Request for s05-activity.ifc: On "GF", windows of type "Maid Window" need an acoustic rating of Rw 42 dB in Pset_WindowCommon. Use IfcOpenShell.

First a look at what the model holds.

```python
import ifcopenshell
import ifcopenshell.util.element

model = ifcopenshell.open("s05-activity.ifc")
print(model.schema)
storey = next(s for s in model.by_type("IfcBuildingStorey") if s.Name == "GF")
windows = [e for e in ifcopenshell.util.element.get_decomposition(storey) if e.is_a("IfcWindow")]
seen = {}
for e in windows:
    element_type = ifcopenshell.util.element.get_type(e)
    key = (element_type.Name if element_type != e and element_type else None, ifcopenshell.util.element.get_pset(e, "Pset_WindowCommon", "AcousticRating"))
    seen[key] = seen.get(key, 0) + 1
for (name, value), count in sorted(seen.items(), key=str):
    print(count, "x", name, "|", value)
```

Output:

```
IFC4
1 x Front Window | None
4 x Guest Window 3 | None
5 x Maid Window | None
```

```python
import ifcopenshell
import ifcopenshell.api.pset
import ifcopenshell.util.element

model = ifcopenshell.open("s05-activity.ifc")

storey = next(s for s in model.by_type("IfcBuildingStorey") if s.Name == "GF")
windows = [e for e in ifcopenshell.util.element.get_decomposition(storey) if e.is_a("IfcWindow")]

count = 0
for e in windows:
    element_type = ifcopenshell.util.element.get_type(e)
    if element_type in (None, e) or element_type.Name != "Maid Window":
        continue
    # add_pset returns the element's existing set when there is one.
    pset = ifcopenshell.api.pset.add_pset(model, product=e, name="Pset_WindowCommon")
    ifcopenshell.api.pset.edit_pset(model, pset=pset, properties={"AcousticRating": "Rw 42 dB"})
    count += 1

print(count, "windows updated")

model.write("s05-activity_edited.ifc")
```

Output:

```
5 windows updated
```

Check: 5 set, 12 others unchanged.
